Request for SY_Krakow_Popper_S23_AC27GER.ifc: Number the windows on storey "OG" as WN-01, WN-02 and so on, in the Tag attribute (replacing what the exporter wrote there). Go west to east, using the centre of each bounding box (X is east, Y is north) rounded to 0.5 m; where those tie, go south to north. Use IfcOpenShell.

First a look at what the model holds.

```python
import ifcopenshell
import ifcopenshell.util.element
import ifcopenshell.util.placement

model = ifcopenshell.open("SY_Krakow_Popper_S23_AC27GER.ifc")
print(model.schema)
storey = next(s for s in model.by_type("IfcBuildingStorey") if s.Name == "OG")
windows = [e for e in ifcopenshell.util.element.get_decomposition(storey) if e.is_a("IfcWindow")]
for e in sorted(windows, key=lambda e: e.id()):
    origin = ifcopenshell.util.placement.get_local_placement(e.ObjectPlacement)[:3, 3]
    print(e.id(), e.Tag, e.Name, origin.round(2) + 0.0, sep=" | ")
```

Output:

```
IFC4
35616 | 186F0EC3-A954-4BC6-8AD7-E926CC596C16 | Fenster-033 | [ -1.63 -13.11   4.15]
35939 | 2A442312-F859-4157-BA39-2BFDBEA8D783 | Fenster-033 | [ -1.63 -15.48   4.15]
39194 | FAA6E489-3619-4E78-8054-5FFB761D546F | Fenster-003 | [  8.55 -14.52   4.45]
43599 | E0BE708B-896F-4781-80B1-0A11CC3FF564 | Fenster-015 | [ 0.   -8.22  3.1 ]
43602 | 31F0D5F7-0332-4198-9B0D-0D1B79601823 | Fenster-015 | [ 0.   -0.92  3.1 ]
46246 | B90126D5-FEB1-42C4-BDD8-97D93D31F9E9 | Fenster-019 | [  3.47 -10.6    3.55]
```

```python
import ifcopenshell
import ifcopenshell.geom
import ifcopenshell.util.element
import ifcopenshell.util.shape

model = ifcopenshell.open("SY_Krakow_Popper_S23_AC27GER.ifc")
settings = ifcopenshell.geom.settings()
settings.set("use-world-coords", True)


def centre(element):
    shape = ifcopenshell.geom.create_shape(settings, element)
    return ifcopenshell.util.shape.get_bbox_centroid(shape.geometry)


storey = next(s for s in model.by_type("IfcBuildingStorey") if s.Name == "OG")
windows = [e for e in ifcopenshell.util.element.get_decomposition(storey) if e.is_a("IfcWindow")]

# Insertion points can sit at a corner or the storey origin, so sort by the geometry (in metres).
centres = {e: centre(e) for e in windows}
windows.sort(key=lambda e: (round(centres[e][0] / 0.5), centres[e][1]))

for i, e in enumerate(windows, start=1):
    number = f"WN-{i:02d}"
    e.Tag = number
    print(e.id(), number)

model.write("SY_Krakow_Popper_S23_AC27GER_rev.ifc")
```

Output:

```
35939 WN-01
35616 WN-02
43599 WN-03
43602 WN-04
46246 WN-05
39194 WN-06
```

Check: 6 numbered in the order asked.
